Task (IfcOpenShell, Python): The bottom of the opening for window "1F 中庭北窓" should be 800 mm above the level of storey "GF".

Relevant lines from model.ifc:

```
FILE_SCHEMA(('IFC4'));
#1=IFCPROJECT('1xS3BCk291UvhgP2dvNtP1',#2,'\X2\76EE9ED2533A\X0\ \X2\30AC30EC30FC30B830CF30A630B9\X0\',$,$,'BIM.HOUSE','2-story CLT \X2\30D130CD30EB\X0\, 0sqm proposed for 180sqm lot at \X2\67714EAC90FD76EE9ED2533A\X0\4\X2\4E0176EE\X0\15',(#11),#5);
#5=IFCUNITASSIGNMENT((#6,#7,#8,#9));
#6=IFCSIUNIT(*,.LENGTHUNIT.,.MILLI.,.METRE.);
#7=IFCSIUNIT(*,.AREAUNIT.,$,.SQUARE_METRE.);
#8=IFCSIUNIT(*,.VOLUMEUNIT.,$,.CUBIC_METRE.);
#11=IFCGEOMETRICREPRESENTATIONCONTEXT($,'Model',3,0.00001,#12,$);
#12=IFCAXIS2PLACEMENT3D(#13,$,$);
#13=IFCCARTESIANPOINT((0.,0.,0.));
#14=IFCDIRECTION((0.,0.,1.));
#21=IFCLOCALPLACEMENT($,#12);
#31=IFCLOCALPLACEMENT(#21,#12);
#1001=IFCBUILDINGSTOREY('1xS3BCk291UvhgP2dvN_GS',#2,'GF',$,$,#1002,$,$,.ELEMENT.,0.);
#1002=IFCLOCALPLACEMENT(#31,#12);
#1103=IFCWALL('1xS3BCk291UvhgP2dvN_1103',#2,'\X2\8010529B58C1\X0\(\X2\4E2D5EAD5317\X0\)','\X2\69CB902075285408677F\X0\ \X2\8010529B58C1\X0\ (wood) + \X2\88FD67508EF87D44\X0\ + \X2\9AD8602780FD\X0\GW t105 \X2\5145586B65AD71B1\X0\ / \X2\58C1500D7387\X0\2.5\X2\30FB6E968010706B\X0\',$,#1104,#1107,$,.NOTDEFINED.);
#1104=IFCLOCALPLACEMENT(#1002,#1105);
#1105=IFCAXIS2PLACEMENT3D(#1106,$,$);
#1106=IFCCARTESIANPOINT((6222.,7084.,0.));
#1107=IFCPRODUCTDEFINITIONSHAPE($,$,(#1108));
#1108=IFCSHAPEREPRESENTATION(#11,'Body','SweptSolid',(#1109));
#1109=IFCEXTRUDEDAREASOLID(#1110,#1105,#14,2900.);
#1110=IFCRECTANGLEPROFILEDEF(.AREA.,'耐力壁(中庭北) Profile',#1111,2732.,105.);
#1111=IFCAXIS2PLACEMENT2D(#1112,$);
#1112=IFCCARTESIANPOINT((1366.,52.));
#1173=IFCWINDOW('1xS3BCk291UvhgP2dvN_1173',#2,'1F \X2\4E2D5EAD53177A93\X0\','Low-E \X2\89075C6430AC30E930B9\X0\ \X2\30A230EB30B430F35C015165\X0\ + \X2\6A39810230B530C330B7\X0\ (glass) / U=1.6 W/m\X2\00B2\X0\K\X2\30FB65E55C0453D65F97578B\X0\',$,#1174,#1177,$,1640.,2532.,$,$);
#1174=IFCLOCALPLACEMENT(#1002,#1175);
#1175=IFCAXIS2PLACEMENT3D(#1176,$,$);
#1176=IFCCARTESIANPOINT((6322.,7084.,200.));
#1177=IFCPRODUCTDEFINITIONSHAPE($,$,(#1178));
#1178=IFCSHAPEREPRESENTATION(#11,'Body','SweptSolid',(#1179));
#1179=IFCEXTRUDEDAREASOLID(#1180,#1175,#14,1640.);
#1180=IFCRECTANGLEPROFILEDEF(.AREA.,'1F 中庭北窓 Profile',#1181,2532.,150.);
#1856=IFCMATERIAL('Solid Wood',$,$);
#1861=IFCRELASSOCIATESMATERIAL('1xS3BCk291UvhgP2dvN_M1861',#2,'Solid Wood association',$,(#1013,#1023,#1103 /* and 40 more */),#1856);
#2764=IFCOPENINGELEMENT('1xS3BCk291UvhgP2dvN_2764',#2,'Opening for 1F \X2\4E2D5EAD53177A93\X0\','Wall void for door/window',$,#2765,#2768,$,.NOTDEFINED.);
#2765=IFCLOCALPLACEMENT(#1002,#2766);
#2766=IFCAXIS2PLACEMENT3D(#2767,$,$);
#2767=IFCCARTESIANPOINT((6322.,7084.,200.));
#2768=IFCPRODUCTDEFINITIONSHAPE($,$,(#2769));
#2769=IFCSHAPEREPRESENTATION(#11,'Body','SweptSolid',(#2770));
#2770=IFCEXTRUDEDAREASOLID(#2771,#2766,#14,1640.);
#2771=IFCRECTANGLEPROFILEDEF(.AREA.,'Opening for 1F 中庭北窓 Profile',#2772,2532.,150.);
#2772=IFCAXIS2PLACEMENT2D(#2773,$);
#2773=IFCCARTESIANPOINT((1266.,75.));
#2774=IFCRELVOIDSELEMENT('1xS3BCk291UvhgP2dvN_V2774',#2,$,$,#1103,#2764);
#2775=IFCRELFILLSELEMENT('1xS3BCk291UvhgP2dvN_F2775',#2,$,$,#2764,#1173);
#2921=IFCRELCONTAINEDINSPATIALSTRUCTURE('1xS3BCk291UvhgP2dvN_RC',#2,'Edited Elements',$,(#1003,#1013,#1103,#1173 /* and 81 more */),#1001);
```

```python
import numpy as np
import ifcopenshell
import ifcopenshell.api.geometry
import ifcopenshell.geom
import ifcopenshell.util.element
import ifcopenshell.util.placement
import ifcopenshell.util.shape
import ifcopenshell.util.unit

model = ifcopenshell.open("model.ifc")
unit_scale = ifcopenshell.util.unit.calculate_unit_scale(model)

window = model.by_id(1173)
opening = window.FillsVoids[0].RelatingOpeningElement
storey = ifcopenshell.util.element.get_container(window, ifc_class="IfcBuildingStorey")
level = ifcopenshell.util.placement.get_local_placement(storey.ObjectPlacement)[2, 3]

# The opening's origin need not be at the sill, so measure its lowest point.
shape = ifcopenshell.geom.create_shape(ifcopenshell.geom.settings(), opening)
bottom = ifcopenshell.util.shape.get_shape_bottom_elevation(shape, shape.geometry) / unit_scale
dz = level + 0.8 / unit_scale - bottom

shift = np.array([0.0, 0.0, dz])
# The window is not placed relative to its opening, so move both.
for product in (opening, window):
    matrix = ifcopenshell.util.placement.get_local_placement(product.ObjectPlacement)
    matrix[:3, 3] += shift
    ifcopenshell.api.geometry.edit_object_placement(model, product=product, matrix=matrix, is_si=False)

print(f"moved by {dz * unit_scale:+.3f} m")

model.write("model_v2.ifc")
```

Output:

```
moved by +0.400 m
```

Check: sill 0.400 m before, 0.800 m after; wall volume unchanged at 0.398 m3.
